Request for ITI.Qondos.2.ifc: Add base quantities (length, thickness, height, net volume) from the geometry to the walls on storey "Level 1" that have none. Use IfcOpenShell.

First a look at what the model holds.

```python
import ifcopenshell
import ifcopenshell.util.element
import ifcopenshell.util.unit

model = ifcopenshell.open("ITI.Qondos.2.ifc")
print(model.schema)
for unit_type in ("LENGTHUNIT", "AREAUNIT", "VOLUMEUNIT"):
    print(unit_type, ifcopenshell.util.unit.calculate_unit_scale(model, unit_type))
storey = next(s for s in model.by_type("IfcBuildingStorey") if s.Name == "Level 1")
walls = [e for e in ifcopenshell.util.element.get_decomposition(storey) if e.is_a("IfcWall")]
for e in sorted(walls, key=lambda e: e.id()):
    print(e.id(), e.is_a(), e.Name, list(ifcopenshell.util.element.get_psets(e, qtos_only=True)), sep=" | ")
```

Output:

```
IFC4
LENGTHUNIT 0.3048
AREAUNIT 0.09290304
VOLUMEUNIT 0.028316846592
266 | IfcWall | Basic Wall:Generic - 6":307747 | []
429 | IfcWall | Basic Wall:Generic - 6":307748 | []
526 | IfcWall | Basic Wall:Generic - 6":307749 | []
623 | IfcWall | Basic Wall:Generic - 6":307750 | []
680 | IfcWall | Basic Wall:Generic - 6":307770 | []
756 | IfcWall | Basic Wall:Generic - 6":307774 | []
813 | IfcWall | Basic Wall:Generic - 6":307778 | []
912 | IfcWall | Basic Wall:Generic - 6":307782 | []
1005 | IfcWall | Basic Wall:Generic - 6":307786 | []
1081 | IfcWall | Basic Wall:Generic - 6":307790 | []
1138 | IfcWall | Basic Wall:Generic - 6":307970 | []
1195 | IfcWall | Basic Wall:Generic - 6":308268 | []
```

```python
import ifcopenshell
import ifcopenshell.api.pset
import ifcopenshell.geom
import ifcopenshell.util.element
import ifcopenshell.util.shape
import ifcopenshell.util.unit

model = ifcopenshell.open("ITI.Qondos.2.ifc")
unit_scale = ifcopenshell.util.unit.calculate_unit_scale(model)
volume_scale = ifcopenshell.util.unit.calculate_unit_scale(model, "VOLUMEUNIT")
settings = ifcopenshell.geom.settings()

storey = next(s for s in model.by_type("IfcBuildingStorey") if s.Name == "Level 1")
walls = [e for e in ifcopenshell.util.element.get_decomposition(storey) if e.is_a("IfcWall")]

for e in sorted(walls, key=lambda e: e.id()):
    if ifcopenshell.util.element.get_psets(e, qtos_only=True, should_inherit=False):
        continue
    # Geometry comes back in metres, in the element's own axes.
    shape = ifcopenshell.geom.create_shape(settings, e)
    values = {
        "Length": ifcopenshell.util.shape.get_x(shape.geometry) / unit_scale,
        "Width": ifcopenshell.util.shape.get_y(shape.geometry) / unit_scale,
        "Height": ifcopenshell.util.shape.get_z(shape.geometry) / unit_scale,
        "NetVolume": ifcopenshell.util.shape.get_volume(shape.geometry) / volume_scale,
    }
    qto = ifcopenshell.api.pset.add_qto(model, product=e, name="Qto_WallBaseQuantities")
    ifcopenshell.api.pset.edit_qto(model, qto=qto, properties=values)
    print(e.id(), {k: round(v, 3) for k, v in values.items()})

model.write("ITI.Qondos.2-out.ifc")
```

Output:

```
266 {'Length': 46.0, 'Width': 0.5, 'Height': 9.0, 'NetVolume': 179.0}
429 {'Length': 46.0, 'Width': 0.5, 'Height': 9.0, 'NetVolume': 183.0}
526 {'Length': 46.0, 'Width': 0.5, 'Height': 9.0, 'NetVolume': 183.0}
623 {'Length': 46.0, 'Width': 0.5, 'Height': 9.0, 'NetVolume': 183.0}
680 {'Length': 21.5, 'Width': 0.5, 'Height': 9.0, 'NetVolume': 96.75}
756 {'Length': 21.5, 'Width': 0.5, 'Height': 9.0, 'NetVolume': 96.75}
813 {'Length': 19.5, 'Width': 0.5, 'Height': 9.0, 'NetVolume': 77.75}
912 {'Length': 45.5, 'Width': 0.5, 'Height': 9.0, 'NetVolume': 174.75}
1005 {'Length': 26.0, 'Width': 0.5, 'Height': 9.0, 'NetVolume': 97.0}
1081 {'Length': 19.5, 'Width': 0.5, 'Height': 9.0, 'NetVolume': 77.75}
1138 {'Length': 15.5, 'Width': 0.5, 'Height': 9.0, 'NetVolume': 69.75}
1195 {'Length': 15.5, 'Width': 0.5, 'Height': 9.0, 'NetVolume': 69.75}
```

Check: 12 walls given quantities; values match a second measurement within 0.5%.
